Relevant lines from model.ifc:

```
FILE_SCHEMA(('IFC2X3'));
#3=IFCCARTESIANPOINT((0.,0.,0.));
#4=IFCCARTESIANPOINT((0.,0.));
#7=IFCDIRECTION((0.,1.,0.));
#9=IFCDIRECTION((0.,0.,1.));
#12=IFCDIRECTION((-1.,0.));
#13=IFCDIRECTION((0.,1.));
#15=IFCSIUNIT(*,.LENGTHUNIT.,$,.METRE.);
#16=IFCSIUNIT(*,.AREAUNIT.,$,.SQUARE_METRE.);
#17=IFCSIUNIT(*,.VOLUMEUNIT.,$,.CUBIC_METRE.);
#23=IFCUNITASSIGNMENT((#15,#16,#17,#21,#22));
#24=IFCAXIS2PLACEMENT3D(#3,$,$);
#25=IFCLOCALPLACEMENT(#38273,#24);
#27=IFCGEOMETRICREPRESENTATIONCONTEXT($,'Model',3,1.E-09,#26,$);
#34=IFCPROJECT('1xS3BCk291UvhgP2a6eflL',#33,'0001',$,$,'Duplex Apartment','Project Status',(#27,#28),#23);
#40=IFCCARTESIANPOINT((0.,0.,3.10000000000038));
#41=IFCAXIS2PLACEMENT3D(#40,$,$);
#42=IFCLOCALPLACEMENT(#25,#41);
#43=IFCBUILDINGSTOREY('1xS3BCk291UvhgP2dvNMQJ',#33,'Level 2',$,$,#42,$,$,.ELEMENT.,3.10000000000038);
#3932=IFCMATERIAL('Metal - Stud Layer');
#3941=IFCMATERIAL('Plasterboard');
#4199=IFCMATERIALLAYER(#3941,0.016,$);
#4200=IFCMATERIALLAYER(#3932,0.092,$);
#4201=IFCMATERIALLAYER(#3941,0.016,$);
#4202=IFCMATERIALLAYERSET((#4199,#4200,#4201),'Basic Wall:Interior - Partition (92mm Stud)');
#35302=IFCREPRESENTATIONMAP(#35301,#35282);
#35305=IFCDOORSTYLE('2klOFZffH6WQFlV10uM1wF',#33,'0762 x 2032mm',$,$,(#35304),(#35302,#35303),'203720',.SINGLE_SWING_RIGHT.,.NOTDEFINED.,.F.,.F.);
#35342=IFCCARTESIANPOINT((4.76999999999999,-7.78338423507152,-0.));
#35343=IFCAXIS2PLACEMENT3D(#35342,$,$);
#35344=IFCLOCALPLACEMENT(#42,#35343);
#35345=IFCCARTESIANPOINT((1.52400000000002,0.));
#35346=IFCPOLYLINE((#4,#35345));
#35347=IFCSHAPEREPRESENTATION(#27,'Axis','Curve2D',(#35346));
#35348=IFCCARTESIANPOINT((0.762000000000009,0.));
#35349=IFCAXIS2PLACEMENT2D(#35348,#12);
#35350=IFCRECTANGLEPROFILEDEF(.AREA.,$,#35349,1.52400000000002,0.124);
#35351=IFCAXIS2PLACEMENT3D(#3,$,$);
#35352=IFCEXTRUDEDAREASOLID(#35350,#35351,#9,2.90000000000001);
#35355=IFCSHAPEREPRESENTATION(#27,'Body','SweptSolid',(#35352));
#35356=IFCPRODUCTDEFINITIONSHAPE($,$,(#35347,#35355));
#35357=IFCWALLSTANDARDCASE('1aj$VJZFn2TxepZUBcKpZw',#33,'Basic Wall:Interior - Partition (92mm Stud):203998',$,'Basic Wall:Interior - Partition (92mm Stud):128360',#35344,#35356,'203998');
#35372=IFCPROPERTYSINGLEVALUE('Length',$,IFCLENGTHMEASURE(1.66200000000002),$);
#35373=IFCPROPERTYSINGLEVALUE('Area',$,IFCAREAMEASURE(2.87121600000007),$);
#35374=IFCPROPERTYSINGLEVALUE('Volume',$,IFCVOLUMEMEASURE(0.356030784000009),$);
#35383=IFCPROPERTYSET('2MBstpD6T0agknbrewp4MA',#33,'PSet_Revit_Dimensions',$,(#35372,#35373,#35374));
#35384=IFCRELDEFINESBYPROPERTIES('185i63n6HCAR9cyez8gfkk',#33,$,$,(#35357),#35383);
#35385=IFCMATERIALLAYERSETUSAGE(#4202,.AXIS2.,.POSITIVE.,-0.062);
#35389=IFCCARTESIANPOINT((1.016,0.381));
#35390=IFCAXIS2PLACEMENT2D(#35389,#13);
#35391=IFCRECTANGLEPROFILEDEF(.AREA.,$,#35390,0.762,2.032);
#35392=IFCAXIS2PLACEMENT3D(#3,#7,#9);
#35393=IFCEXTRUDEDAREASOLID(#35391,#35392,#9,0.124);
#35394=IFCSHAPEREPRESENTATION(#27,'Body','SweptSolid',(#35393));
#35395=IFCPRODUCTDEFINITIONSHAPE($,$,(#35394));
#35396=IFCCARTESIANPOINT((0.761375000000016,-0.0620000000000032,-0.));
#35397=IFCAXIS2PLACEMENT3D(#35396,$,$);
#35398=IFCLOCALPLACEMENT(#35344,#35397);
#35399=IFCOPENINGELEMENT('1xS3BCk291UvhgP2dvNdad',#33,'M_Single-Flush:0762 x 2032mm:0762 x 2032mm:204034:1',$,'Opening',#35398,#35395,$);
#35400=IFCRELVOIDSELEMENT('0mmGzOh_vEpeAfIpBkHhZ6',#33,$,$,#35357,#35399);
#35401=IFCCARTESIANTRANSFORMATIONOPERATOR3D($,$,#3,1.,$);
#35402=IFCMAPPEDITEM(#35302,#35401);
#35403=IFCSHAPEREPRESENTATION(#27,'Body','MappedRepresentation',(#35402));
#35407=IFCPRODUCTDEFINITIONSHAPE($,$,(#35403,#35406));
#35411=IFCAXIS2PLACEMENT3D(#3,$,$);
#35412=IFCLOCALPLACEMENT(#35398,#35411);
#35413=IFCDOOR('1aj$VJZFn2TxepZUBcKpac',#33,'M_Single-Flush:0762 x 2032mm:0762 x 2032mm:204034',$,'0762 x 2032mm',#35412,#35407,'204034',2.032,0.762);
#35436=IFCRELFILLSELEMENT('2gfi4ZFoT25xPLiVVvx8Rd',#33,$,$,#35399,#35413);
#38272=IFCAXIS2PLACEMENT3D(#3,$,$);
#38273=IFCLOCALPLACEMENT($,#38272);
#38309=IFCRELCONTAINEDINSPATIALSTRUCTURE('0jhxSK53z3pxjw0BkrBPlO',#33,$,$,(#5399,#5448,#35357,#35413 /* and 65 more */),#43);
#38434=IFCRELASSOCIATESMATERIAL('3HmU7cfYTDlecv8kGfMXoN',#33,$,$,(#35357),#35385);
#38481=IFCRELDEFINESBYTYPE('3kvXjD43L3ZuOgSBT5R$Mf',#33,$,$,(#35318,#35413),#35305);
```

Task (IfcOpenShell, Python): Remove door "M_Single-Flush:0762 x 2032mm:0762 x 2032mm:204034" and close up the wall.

```python
import ifcopenshell
import ifcopenshell.api.feature
import ifcopenshell.api.pset
import ifcopenshell.api.root
import ifcopenshell.geom
import ifcopenshell.util.element
import ifcopenshell.util.shape
import ifcopenshell.util.unit

model = ifcopenshell.open("model.ifc")
area_scale = ifcopenshell.util.unit.calculate_unit_scale(model, "AREAUNIT")
volume_scale = ifcopenshell.util.unit.calculate_unit_scale(model, "VOLUMEUNIT")
settings = ifcopenshell.geom.settings()


def volume(element):
    """Net volume in cubic metres, openings subtracted."""
    shape = ifcopenshell.geom.create_shape(settings, element)
    return ifcopenshell.util.shape.get_volume(shape.geometry)


door = model.by_guid("1aj$VJZFn2TxepZUBcKpac")
opening = door.FillsVoids[0].RelatingOpeningElement
wall = opening.VoidsElements[0].RelatingBuildingElement
before = volume(wall)

ifcopenshell.api.root.remove_product(model, product=door)
ifcopenshell.api.feature.remove_feature(model, feature=opening)

after = volume(wall)
thickness = 0.124  # wall thickness in metres

# Update the wall's stored quantities.
pset = model.by_id(ifcopenshell.util.element.get_pset(wall, "PSet_Revit_Dimensions", should_inherit=False)["id"])
ifcopenshell.api.pset.edit_pset(model, pset=pset, properties={
    "Area": model.create_entity("IfcAreaMeasure", after / thickness / area_scale),
    "Volume": model.create_entity("IfcVolumeMeasure", after / volume_scale),
})

print(f"wall volume {before:.3f} -> {after:.3f} m3")

model.write("model_v2.ifc")
```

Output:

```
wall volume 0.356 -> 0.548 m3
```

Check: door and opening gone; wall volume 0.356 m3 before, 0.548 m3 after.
